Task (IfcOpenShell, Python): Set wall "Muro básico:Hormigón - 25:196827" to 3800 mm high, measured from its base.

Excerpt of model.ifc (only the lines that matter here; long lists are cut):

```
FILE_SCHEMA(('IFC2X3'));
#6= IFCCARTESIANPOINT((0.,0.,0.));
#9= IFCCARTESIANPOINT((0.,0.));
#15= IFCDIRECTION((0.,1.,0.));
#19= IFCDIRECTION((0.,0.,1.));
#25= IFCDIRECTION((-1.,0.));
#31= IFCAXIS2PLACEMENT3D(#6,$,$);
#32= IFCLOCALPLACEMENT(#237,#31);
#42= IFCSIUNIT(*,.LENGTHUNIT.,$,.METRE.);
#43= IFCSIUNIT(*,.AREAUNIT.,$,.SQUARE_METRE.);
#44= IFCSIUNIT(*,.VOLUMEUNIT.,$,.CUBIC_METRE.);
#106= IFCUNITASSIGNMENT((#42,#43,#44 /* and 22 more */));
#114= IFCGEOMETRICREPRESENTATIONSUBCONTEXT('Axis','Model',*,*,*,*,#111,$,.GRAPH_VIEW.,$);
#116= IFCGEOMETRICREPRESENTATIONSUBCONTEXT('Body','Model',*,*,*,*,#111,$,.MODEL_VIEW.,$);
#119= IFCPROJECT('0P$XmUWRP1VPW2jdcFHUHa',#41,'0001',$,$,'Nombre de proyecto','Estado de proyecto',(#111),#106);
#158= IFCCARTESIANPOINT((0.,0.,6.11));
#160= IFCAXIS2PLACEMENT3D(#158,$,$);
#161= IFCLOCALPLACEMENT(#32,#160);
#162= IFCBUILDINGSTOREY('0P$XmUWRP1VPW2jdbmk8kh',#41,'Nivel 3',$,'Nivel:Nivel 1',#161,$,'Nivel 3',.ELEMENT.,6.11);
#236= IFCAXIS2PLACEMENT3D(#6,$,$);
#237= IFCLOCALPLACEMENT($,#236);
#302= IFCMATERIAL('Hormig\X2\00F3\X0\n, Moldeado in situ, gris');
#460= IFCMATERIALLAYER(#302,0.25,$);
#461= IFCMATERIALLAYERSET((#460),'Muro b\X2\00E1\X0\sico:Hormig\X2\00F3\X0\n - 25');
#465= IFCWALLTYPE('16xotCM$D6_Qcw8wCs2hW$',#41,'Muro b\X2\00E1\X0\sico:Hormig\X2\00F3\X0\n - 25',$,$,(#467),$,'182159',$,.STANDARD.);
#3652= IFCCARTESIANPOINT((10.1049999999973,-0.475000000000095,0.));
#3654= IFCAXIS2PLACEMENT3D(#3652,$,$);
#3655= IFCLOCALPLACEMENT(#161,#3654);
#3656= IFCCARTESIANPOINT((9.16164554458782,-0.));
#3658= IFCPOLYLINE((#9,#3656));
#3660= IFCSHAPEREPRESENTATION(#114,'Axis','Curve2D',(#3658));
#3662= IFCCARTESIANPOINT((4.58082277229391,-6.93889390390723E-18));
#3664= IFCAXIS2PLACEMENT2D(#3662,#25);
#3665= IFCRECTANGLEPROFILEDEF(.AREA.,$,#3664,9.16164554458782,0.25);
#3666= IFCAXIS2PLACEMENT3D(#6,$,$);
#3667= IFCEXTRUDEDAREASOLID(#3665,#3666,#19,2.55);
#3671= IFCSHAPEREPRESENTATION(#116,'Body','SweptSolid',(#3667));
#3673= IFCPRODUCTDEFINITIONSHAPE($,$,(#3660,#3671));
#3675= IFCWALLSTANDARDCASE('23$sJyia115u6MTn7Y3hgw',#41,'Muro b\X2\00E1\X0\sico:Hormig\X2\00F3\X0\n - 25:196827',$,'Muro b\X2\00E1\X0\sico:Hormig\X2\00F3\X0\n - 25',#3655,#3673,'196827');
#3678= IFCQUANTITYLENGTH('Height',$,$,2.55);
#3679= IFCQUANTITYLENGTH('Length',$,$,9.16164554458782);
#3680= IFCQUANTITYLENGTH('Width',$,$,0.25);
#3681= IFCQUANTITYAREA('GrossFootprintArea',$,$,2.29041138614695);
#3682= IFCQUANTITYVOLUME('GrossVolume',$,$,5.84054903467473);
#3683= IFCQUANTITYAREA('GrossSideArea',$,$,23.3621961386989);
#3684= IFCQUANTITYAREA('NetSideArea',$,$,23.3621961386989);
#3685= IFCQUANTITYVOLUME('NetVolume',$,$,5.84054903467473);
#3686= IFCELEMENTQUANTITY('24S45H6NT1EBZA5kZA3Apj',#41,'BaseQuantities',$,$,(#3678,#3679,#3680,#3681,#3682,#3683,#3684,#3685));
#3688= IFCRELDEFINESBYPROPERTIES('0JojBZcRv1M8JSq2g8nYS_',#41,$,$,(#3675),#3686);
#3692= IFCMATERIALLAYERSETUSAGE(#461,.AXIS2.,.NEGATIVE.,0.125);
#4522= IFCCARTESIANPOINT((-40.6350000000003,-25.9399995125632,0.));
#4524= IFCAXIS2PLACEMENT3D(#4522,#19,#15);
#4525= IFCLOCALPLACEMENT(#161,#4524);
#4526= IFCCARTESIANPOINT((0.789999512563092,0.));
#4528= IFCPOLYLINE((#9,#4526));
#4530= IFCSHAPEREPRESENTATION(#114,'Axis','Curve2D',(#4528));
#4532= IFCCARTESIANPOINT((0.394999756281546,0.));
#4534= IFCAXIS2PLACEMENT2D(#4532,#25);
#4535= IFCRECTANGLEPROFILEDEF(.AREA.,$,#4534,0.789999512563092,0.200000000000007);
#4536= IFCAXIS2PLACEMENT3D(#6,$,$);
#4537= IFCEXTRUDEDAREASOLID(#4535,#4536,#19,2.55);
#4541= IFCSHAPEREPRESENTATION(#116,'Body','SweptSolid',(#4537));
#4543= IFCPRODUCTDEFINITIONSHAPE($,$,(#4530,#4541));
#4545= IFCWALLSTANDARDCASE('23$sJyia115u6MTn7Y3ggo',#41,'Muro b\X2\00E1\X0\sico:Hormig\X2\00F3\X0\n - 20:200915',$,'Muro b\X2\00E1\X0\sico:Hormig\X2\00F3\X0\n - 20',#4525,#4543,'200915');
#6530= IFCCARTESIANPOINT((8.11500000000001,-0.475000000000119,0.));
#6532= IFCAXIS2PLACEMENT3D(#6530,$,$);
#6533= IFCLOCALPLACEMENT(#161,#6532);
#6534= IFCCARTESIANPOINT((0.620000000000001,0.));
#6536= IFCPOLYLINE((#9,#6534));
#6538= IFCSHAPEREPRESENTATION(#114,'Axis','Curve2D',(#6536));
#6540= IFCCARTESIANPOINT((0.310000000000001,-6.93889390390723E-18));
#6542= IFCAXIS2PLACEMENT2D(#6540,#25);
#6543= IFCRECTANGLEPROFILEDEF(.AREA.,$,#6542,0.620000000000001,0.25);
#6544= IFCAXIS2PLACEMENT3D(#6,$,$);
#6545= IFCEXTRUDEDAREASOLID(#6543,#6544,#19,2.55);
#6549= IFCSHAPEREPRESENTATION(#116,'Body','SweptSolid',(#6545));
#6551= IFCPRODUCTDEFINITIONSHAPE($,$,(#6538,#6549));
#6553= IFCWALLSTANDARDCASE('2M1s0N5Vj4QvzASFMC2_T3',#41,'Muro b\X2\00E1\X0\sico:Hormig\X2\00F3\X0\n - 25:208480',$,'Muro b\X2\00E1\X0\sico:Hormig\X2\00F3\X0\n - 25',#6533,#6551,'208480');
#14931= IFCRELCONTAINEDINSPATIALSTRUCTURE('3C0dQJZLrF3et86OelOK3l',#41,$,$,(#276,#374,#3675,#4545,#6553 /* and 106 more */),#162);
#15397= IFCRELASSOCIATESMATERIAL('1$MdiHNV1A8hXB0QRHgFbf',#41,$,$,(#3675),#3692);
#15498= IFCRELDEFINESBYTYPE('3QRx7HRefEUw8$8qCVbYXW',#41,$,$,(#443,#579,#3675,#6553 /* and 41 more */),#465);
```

```python
import ifcopenshell
import ifcopenshell.api.pset
import ifcopenshell.geom
import ifcopenshell.util.element
import ifcopenshell.util.representation
import ifcopenshell.util.shape
import ifcopenshell.util.unit

model = ifcopenshell.open("model.ifc")
unit_scale = ifcopenshell.util.unit.calculate_unit_scale(model)
area_scale = ifcopenshell.util.unit.calculate_unit_scale(model, "AREAUNIT")
volume_scale = ifcopenshell.util.unit.calculate_unit_scale(model, "VOLUMEUNIT")
settings = ifcopenshell.geom.settings()


def volume(element):
    """Net volume in cubic metres, openings subtracted."""
    shape = ifcopenshell.geom.create_shape(settings, element)
    return ifcopenshell.util.shape.get_volume(shape.geometry)


wall = model.by_guid("23$sJyia115u6MTn7Y3hgw")
before = volume(wall)

body = ifcopenshell.util.representation.get_representation(wall, "Model", "Body")
solid = body.Items[0]
old_height = solid.Depth
solid.Depth = 3.8 / unit_scale
after = volume(wall)
thickness = 0.25  # wall thickness in metres

# Update the stored height, areas and volumes.
qto = model.by_id(ifcopenshell.util.element.get_pset(wall, "BaseQuantities", should_inherit=False)["id"])
ifcopenshell.api.pset.edit_qto(model, qto=qto, properties={
    "Height": solid.Depth,
    "GrossVolume": ifcopenshell.util.element.get_pset(wall, "BaseQuantities", "GrossVolume") * solid.Depth / old_height,
    "GrossSideArea": ifcopenshell.util.element.get_pset(wall, "BaseQuantities", "GrossSideArea") * solid.Depth / old_height,
    "NetSideArea": after / thickness / area_scale,
    "NetVolume": after / volume_scale,
})

print(f"height {old_height:g} -> {solid.Depth:g}, volume {before:.3f} -> {after:.3f} m3")

model.write("model_v2.ifc")
```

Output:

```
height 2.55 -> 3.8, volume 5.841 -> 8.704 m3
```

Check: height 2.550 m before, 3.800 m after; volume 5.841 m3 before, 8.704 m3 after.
